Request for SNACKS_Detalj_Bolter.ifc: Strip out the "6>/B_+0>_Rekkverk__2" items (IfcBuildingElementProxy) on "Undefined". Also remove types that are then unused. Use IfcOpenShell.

First a look at what the model holds.

```python
import ifcopenshell
import ifcopenshell.util.element

model = ifcopenshell.open("SNACKS_Detalj_Bolter.ifc")
print(model.schema)
storey = next(s for s in model.by_type("IfcBuildingStorey") if s.Name == "Undefined")
proxies = [e for e in ifcopenshell.util.element.get_decomposition(storey) if e.is_a("IfcBuildingElementProxy")]
seen = {}
for e in proxies:
    element_type = ifcopenshell.util.element.get_type(e)
    name = element_type.Name if element_type not in (None, e) else None
    seen[name] = seen.get(name, 0) + 1
for name, count in sorted(seen.items(), key=str):
    print(count, "x", name)
```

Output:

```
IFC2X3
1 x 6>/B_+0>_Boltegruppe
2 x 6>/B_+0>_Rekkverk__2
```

```python
import ifcopenshell
import ifcopenshell.api.root
import ifcopenshell.util.element

model = ifcopenshell.open("SNACKS_Detalj_Bolter.ifc")

storey = next(s for s in model.by_type("IfcBuildingStorey") if s.Name == "Undefined")
proxies = [e for e in ifcopenshell.util.element.get_decomposition(storey) if e.is_a("IfcBuildingElementProxy")]
targets = [e for e in proxies if (t := ifcopenshell.util.element.get_type(e)) not in (None, e) and t.Name == "6>/B_+0>_Rekkverk__2"]
types = {ifcopenshell.util.element.get_type(e) for e in targets} - {None, *targets}

for e in targets:
    ifcopenshell.api.root.remove_product(model, product=e)
print(len(targets), "removed")

unused = [t for t in types if not ifcopenshell.util.element.get_types(t)]
for t in unused:
    ifcopenshell.api.root.remove_product(model, product=t)
print(len(unused), "unused types removed")

model.write("SNACKS_Detalj_Bolter_updated.ifc")
```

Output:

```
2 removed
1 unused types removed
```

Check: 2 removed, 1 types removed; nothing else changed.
